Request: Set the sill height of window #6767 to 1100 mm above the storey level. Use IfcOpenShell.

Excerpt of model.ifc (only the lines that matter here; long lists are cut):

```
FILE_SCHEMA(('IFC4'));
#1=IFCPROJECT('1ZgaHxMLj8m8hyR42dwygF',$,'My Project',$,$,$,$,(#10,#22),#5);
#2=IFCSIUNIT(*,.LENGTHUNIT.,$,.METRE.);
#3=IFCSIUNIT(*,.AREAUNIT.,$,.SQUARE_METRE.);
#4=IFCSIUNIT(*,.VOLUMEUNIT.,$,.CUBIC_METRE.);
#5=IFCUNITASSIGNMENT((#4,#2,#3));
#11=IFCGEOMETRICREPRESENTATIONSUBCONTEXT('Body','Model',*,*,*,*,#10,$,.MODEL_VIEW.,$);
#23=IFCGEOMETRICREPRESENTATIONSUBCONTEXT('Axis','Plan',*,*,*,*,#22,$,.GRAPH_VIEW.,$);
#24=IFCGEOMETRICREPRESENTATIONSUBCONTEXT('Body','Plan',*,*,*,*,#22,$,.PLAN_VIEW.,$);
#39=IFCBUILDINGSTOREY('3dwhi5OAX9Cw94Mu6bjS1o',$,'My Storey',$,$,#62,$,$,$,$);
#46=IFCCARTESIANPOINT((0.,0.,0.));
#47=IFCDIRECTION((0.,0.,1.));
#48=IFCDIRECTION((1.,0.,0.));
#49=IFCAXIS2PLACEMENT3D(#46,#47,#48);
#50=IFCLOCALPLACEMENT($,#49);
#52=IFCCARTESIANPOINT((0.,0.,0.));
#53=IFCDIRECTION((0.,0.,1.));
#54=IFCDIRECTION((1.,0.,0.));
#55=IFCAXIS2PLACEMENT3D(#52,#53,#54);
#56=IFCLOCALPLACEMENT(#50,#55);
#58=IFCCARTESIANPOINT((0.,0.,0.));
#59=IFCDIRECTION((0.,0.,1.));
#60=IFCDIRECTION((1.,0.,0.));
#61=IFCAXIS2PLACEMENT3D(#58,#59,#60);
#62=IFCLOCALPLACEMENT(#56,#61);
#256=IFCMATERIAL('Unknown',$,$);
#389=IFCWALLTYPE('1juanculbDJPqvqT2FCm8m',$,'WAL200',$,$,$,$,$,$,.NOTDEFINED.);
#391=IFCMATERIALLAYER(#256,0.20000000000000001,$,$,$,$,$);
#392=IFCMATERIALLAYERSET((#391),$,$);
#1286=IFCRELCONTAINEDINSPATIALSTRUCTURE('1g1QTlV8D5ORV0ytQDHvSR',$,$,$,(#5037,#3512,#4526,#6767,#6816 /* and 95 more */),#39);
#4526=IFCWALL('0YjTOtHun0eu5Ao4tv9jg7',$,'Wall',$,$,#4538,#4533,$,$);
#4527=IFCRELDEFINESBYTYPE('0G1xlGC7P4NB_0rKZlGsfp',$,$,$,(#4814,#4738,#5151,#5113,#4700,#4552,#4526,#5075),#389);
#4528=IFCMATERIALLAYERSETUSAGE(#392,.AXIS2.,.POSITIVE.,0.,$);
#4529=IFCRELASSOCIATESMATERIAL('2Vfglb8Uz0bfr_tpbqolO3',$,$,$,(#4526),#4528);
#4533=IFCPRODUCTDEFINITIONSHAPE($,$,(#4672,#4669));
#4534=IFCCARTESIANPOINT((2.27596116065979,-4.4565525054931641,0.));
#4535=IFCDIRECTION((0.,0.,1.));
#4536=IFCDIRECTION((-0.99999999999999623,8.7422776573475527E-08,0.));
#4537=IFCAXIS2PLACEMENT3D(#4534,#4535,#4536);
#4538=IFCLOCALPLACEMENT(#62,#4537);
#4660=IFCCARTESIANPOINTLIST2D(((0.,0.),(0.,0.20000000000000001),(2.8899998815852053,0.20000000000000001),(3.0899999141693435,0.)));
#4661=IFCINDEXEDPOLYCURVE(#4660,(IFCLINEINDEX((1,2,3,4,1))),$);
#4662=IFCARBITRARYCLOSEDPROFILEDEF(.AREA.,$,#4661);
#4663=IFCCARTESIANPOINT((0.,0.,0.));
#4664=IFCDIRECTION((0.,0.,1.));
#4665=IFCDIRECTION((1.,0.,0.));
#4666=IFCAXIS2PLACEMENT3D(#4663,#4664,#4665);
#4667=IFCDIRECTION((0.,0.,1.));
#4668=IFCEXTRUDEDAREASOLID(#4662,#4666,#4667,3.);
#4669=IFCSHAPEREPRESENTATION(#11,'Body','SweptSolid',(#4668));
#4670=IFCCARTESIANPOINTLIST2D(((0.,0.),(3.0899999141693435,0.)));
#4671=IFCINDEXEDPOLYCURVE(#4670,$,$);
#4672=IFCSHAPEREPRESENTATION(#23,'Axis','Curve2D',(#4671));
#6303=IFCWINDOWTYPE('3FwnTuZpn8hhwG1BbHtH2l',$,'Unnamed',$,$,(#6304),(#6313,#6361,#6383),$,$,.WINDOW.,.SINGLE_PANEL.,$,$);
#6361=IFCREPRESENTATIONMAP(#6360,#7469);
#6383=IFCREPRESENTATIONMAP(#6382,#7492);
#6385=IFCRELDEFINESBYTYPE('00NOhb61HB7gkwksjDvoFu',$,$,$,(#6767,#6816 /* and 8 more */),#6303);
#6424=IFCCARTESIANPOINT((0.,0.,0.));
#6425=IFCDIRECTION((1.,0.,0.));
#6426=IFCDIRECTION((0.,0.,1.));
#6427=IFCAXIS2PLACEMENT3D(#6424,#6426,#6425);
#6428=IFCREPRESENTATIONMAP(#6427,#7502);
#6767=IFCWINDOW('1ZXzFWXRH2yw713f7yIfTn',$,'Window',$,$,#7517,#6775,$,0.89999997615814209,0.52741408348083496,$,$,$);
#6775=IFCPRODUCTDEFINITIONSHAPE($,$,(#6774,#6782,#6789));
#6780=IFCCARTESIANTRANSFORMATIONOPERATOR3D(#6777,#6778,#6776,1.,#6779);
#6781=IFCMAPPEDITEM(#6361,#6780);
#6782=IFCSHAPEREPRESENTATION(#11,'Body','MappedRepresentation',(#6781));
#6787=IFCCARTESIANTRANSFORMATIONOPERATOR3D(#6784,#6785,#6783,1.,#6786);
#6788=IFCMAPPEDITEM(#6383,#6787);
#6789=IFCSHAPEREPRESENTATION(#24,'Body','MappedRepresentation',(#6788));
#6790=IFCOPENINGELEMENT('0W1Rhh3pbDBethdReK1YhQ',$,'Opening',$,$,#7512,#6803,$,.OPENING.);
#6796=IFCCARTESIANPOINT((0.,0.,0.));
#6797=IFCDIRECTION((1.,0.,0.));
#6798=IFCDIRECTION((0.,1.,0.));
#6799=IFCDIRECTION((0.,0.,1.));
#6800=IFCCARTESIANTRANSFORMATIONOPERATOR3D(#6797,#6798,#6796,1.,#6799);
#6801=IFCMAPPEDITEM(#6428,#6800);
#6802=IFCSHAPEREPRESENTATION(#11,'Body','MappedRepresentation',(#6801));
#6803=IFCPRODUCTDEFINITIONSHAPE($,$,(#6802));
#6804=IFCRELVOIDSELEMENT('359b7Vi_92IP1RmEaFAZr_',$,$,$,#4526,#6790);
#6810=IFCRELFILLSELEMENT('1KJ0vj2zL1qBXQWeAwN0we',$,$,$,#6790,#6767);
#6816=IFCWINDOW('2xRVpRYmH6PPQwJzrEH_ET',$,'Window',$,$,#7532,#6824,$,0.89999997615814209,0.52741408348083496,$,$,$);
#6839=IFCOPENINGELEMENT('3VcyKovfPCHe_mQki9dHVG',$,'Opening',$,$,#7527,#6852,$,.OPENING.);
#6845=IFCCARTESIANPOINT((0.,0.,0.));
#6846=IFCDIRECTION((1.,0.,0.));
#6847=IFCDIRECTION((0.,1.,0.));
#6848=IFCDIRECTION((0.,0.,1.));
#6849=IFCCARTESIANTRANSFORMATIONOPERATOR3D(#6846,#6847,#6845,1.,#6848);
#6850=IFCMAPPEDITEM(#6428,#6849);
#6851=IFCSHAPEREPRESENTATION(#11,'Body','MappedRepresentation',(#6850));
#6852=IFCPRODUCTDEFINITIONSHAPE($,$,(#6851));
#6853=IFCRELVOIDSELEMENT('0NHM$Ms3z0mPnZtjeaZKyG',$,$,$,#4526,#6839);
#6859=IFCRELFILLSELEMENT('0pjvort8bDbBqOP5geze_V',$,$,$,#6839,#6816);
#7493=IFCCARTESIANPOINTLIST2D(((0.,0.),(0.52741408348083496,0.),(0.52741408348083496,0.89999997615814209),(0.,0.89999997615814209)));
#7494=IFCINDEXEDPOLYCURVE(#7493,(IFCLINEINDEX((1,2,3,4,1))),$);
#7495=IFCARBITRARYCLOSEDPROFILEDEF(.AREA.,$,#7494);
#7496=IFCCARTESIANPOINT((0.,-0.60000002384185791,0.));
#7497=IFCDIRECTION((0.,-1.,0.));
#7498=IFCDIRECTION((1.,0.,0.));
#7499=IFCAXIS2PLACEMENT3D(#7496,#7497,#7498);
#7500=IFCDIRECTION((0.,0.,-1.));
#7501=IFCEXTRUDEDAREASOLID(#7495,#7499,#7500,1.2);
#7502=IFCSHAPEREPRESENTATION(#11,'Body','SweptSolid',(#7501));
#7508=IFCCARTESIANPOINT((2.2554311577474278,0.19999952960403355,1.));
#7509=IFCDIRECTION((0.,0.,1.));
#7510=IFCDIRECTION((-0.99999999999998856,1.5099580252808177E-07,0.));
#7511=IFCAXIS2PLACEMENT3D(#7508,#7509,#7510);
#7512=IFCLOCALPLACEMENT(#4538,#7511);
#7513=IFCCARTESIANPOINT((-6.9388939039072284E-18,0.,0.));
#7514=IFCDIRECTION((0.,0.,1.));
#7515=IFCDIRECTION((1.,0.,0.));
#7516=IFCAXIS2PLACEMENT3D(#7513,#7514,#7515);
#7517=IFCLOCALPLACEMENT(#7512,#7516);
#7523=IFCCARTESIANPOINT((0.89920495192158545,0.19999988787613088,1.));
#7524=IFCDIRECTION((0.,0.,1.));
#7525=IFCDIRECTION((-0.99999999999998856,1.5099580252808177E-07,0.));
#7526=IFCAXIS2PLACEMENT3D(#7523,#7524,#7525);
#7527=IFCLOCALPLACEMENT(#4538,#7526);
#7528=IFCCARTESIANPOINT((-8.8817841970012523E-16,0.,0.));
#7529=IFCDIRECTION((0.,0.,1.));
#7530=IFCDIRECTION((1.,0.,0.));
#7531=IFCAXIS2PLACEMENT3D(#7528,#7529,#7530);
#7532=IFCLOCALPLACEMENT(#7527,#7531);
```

```python
import numpy as np
import ifcopenshell
import ifcopenshell.api.geometry
import ifcopenshell.geom
import ifcopenshell.util.element
import ifcopenshell.util.placement
import ifcopenshell.util.shape
import ifcopenshell.util.unit

model = ifcopenshell.open("model.ifc")
unit_scale = ifcopenshell.util.unit.calculate_unit_scale(model)

window = model.by_guid("1ZXzFWXRH2yw713f7yIfTn")
opening = window.FillsVoids[0].RelatingOpeningElement
storey = ifcopenshell.util.element.get_container(window, ifc_class="IfcBuildingStorey")
level = ifcopenshell.util.placement.get_local_placement(storey.ObjectPlacement)[2, 3]

# The opening's origin need not be at the sill, so measure its lowest point.
shape = ifcopenshell.geom.create_shape(ifcopenshell.geom.settings(), opening)
bottom = ifcopenshell.util.shape.get_shape_bottom_elevation(shape, shape.geometry) / unit_scale
dz = level + 1.1 / unit_scale - bottom

shift = np.array([0.0, 0.0, dz])
# The window is placed relative to its opening, so it follows when the opening moves.
matrix = ifcopenshell.util.placement.get_local_placement(opening.ObjectPlacement)
matrix[:3, 3] += shift
ifcopenshell.api.geometry.edit_object_placement(
    model, product=opening, matrix=matrix, is_si=False, should_transform_children=True
)

print(f"moved by {dz * unit_scale:+.3f} m")

model.write("model_edited.ifc")
```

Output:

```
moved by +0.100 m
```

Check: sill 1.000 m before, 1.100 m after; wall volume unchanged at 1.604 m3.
